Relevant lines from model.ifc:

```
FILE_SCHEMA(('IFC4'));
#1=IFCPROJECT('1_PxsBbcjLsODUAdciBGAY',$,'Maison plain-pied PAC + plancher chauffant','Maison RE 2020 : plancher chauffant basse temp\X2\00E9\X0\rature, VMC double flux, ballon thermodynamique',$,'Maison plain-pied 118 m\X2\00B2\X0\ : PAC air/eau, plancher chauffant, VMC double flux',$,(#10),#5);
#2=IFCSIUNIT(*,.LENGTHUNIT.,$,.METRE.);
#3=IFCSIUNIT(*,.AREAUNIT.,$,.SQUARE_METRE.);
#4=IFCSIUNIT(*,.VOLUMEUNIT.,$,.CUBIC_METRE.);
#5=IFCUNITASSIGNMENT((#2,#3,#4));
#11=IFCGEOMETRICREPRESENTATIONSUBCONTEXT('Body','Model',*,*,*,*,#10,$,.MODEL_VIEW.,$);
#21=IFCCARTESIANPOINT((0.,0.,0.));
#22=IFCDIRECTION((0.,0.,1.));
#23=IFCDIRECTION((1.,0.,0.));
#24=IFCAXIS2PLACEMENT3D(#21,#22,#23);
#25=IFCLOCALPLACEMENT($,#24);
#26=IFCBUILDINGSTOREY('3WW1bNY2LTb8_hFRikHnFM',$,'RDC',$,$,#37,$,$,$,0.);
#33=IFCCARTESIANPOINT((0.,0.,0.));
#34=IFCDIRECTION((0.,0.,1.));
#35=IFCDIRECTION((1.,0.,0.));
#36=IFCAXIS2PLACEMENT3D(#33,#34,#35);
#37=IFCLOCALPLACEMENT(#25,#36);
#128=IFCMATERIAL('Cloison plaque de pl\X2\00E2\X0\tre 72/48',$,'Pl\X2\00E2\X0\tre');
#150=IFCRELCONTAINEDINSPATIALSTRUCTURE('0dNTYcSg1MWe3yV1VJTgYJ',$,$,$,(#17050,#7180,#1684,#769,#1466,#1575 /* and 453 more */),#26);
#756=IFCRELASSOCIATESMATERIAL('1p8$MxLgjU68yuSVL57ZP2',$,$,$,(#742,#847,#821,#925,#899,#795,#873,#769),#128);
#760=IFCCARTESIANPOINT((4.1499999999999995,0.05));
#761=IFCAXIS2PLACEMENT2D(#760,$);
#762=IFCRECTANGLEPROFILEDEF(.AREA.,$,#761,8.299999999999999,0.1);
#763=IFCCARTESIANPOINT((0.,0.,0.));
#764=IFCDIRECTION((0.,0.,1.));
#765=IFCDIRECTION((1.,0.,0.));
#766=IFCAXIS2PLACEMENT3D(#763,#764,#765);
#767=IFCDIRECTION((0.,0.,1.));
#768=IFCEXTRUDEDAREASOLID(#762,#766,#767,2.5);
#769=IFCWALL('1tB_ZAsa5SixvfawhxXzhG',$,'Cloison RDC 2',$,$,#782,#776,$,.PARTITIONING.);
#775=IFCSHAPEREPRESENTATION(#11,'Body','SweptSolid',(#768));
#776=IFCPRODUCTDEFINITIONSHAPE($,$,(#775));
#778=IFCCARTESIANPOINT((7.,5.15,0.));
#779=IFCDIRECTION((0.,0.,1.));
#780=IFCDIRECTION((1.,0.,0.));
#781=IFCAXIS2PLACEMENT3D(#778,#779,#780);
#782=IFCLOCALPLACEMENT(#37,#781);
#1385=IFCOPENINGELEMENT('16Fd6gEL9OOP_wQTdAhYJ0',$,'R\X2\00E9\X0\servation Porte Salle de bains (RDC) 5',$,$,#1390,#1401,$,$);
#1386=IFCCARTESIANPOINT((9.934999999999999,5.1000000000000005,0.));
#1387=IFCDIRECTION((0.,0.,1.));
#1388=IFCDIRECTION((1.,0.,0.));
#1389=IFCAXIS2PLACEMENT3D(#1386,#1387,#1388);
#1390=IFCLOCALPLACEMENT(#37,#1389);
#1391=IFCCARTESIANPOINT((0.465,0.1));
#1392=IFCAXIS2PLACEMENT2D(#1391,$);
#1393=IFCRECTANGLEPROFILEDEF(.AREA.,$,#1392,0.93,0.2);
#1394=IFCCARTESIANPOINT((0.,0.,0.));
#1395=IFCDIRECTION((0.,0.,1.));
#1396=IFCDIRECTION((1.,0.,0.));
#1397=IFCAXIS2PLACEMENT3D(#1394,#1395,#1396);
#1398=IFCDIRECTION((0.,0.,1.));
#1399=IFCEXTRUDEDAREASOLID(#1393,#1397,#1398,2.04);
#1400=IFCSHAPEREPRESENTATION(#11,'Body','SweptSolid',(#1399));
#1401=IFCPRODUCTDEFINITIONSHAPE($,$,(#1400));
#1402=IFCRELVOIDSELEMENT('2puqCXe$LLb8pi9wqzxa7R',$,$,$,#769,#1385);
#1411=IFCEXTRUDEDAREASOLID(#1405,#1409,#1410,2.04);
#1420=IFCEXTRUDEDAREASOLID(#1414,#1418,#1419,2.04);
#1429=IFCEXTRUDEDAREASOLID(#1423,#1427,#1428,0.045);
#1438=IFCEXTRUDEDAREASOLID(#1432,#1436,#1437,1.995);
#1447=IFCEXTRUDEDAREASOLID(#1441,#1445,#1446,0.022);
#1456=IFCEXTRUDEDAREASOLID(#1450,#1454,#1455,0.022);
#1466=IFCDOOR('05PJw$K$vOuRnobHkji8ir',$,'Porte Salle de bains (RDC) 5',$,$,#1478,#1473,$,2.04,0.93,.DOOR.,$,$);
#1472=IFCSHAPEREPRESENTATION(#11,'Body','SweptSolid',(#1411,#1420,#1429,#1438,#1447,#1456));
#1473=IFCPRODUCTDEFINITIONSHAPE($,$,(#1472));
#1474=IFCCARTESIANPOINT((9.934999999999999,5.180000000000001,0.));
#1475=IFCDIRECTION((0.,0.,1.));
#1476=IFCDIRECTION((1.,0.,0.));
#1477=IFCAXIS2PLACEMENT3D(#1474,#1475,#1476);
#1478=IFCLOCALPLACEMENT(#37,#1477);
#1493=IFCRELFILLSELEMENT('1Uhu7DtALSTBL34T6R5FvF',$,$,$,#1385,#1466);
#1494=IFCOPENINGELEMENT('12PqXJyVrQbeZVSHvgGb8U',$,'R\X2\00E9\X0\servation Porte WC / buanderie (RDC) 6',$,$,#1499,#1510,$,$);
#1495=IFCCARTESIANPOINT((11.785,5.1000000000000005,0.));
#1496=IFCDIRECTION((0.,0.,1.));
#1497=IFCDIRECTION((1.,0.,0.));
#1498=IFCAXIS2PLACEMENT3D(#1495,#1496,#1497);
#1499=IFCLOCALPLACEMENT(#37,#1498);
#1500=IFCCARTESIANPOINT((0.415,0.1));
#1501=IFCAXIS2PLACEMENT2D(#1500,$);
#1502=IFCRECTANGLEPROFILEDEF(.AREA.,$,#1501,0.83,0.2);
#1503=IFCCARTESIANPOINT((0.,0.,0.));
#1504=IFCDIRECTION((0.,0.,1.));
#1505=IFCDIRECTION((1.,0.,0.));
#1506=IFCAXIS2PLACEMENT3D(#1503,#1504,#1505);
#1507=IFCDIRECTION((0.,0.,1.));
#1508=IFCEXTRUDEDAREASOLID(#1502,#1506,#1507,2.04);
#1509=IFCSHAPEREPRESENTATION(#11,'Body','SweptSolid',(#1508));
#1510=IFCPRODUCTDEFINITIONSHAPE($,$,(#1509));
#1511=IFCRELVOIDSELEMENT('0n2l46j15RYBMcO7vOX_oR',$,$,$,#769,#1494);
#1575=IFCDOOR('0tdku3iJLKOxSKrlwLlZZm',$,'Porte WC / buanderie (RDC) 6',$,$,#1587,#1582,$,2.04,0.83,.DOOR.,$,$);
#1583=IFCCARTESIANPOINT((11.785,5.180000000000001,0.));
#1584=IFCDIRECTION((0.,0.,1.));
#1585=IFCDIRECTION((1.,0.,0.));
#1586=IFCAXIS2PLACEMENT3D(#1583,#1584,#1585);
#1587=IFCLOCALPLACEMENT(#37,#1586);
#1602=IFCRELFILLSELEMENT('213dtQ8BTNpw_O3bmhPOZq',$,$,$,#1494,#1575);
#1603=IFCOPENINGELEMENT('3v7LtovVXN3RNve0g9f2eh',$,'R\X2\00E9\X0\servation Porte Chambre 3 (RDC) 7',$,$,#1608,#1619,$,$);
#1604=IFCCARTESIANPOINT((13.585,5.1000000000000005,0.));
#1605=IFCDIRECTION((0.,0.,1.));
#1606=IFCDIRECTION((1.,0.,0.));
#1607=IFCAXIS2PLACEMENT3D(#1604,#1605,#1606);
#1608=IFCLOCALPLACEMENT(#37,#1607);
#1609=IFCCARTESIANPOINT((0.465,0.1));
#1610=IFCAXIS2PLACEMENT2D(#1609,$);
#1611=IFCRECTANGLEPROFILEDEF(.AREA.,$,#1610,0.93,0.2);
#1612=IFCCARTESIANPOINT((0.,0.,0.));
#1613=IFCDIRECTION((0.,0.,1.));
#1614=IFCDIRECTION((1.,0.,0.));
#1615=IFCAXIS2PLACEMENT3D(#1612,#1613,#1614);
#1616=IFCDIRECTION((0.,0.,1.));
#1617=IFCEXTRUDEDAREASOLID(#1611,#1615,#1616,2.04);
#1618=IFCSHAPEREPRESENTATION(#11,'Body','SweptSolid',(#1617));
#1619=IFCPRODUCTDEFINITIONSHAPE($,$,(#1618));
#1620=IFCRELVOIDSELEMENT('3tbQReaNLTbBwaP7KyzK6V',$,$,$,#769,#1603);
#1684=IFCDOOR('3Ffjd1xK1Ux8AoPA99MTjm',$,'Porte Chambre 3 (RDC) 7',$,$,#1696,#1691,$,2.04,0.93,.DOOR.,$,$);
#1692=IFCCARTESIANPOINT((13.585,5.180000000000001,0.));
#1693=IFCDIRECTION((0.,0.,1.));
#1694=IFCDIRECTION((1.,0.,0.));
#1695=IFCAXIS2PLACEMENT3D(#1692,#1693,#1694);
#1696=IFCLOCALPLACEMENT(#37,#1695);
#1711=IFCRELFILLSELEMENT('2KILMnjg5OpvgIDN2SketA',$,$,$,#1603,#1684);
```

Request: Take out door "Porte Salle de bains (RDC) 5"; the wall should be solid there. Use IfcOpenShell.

```python
import ifcopenshell
import ifcopenshell.api.feature
import ifcopenshell.api.root
import ifcopenshell.geom
import ifcopenshell.util.shape

model = ifcopenshell.open("model.ifc")
settings = ifcopenshell.geom.settings()


def volume(element):
    """Net volume in cubic metres, openings subtracted."""
    shape = ifcopenshell.geom.create_shape(settings, element)
    return ifcopenshell.util.shape.get_volume(shape.geometry)


door = model.by_guid("05PJw$K$vOuRnobHkji8ir")
opening = door.FillsVoids[0].RelatingOpeningElement
wall = opening.VoidsElements[0].RelatingBuildingElement
before = volume(wall)

ifcopenshell.api.root.remove_product(model, product=door)
ifcopenshell.api.feature.remove_feature(model, feature=opening)

after = volume(wall)

print(f"wall volume {before:.3f} -> {after:.3f} m3")

model.write("model_rev.ifc")
```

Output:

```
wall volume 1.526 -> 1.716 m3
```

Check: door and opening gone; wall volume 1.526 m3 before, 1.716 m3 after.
